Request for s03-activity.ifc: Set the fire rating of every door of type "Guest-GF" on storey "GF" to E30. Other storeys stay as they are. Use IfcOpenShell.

First a look at what the model holds.

```python
import ifcopenshell
import ifcopenshell.util.element

model = ifcopenshell.open("s03-activity.ifc")
print(model.schema)
storey = next(s for s in model.by_type("IfcBuildingStorey") if s.Name == "GF")
doors = [e for e in ifcopenshell.util.element.get_decomposition(storey) if e.is_a("IfcDoor")]
seen = {}
for e in doors:
    element_type = ifcopenshell.util.element.get_type(e)
    key = (element_type.Name if element_type != e and element_type else None, ifcopenshell.util.element.get_pset(e, "Pset_DoorCommon", "FireRating"))
    seen[key] = seen.get(key, 0) + 1
for (name, value), count in sorted(seen.items(), key=str):
    print(count, "x", name, "|", value)
```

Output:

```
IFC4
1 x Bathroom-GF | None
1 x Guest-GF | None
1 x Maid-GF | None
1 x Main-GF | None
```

```python
import ifcopenshell
import ifcopenshell.api.pset
import ifcopenshell.util.element

model = ifcopenshell.open("s03-activity.ifc")

storey = next(s for s in model.by_type("IfcBuildingStorey") if s.Name == "GF")
doors = [e for e in ifcopenshell.util.element.get_decomposition(storey) if e.is_a("IfcDoor")]

count = 0
for e in doors:
    element_type = ifcopenshell.util.element.get_type(e)
    if element_type in (None, e) or element_type.Name != "Guest-GF":
        continue
    # add_pset returns the element's existing set when there is one.
    pset = ifcopenshell.api.pset.add_pset(model, product=e, name="Pset_DoorCommon")
    ifcopenshell.api.pset.edit_pset(model, pset=pset, properties={"FireRating": "E30"})
    count += 1

print(count, "doors updated")

model.write("s03-activity-out.ifc")
```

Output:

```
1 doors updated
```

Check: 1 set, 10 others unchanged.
